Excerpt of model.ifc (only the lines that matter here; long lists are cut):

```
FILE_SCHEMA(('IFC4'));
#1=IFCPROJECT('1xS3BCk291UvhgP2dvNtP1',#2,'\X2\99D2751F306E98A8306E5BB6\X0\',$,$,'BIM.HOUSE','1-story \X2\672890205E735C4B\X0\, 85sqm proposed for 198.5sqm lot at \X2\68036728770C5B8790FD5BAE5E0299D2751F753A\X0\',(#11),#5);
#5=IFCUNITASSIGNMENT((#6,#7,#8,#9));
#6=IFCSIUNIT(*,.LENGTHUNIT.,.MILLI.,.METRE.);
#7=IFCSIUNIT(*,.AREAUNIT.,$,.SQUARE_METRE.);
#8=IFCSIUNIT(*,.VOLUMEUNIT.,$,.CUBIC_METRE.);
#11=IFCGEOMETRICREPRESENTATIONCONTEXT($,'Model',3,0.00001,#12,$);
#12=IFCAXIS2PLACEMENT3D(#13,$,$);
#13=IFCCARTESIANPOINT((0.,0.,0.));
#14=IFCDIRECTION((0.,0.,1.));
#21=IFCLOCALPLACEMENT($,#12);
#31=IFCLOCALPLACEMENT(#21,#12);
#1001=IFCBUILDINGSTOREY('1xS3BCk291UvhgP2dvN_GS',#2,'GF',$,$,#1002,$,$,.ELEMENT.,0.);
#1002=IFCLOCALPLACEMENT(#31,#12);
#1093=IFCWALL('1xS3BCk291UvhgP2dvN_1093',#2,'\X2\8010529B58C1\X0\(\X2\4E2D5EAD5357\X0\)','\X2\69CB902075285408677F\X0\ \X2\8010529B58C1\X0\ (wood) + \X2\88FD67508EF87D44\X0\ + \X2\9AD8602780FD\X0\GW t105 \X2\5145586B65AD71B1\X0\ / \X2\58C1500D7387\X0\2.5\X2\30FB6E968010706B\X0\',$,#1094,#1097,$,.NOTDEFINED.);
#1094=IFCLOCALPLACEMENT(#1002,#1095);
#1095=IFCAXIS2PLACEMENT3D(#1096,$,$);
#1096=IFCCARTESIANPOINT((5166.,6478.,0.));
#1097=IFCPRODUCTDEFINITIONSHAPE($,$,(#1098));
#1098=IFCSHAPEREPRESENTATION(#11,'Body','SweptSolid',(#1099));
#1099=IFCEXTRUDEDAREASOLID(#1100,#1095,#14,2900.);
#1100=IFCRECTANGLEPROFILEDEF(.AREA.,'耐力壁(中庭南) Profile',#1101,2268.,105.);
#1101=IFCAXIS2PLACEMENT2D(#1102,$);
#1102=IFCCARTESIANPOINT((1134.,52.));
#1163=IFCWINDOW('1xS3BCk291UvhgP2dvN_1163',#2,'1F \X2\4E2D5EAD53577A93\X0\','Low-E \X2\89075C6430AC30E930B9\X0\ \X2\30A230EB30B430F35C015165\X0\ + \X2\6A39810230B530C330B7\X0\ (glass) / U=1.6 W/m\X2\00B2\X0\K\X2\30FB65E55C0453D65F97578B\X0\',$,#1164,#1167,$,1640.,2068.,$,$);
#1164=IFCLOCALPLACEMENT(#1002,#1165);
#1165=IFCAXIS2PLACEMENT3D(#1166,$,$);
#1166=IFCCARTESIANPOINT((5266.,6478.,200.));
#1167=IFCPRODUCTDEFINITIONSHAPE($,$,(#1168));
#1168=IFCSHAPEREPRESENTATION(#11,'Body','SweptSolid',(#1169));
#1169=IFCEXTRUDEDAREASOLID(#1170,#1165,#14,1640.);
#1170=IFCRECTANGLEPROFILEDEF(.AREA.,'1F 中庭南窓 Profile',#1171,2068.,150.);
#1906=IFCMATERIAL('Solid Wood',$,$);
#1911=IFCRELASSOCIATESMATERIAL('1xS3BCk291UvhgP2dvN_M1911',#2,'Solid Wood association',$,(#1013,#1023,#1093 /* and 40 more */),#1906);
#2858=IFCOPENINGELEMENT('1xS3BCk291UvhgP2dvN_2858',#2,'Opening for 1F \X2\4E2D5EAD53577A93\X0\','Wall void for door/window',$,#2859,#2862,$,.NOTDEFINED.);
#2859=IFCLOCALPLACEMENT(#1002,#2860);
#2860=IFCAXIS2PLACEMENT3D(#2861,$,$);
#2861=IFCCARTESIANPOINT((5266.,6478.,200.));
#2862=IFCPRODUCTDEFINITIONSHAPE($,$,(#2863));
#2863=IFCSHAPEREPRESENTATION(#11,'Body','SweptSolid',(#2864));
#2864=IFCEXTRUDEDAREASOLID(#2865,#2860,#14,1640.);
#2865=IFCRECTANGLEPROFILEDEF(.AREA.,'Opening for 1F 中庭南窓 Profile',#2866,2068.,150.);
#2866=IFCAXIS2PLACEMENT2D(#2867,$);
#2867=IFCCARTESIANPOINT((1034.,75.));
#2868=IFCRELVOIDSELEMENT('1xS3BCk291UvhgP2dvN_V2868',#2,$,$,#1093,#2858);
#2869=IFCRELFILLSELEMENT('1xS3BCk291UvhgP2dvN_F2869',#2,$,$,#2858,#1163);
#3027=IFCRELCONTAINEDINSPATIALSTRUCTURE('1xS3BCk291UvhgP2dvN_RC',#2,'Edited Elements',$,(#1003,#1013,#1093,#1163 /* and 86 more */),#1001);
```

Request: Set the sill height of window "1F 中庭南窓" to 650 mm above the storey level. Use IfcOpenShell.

```python
import numpy as np
import ifcopenshell
import ifcopenshell.api.geometry
import ifcopenshell.geom
import ifcopenshell.util.element
import ifcopenshell.util.placement
import ifcopenshell.util.shape
import ifcopenshell.util.unit

model = ifcopenshell.open("model.ifc")
unit_scale = ifcopenshell.util.unit.calculate_unit_scale(model)

window = model.by_guid("1xS3BCk291UvhgP2dvN_1163")
opening = window.FillsVoids[0].RelatingOpeningElement
storey = ifcopenshell.util.element.get_container(window, ifc_class="IfcBuildingStorey")
level = ifcopenshell.util.placement.get_local_placement(storey.ObjectPlacement)[2, 3]

# The opening's origin need not be at the sill, so measure its lowest point.
shape = ifcopenshell.geom.create_shape(ifcopenshell.geom.settings(), opening)
bottom = ifcopenshell.util.shape.get_shape_bottom_elevation(shape, shape.geometry) / unit_scale
dz = level + 650.0 - bottom

shift = np.array([0.0, 0.0, dz])
# The window is not placed relative to its opening, so move both.
for product in (opening, window):
    matrix = ifcopenshell.util.placement.get_local_placement(product.ObjectPlacement)
    matrix[:3, 3] += shift
    ifcopenshell.api.geometry.edit_object_placement(model, product=product, matrix=matrix, is_si=False)

print(f"moved by {dz * unit_scale:+.3f} m")

model.write("model_edited.ifc")
```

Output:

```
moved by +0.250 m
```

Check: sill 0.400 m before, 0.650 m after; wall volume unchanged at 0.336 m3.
